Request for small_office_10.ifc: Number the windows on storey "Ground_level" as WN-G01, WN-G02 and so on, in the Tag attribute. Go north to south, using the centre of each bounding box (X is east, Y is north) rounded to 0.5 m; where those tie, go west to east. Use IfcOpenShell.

First a look at what the model holds.

```python
import ifcopenshell
import ifcopenshell.util.element
import ifcopenshell.util.placement

model = ifcopenshell.open("small_office_10.ifc")
print(model.schema)
storey = next(s for s in model.by_type("IfcBuildingStorey") if s.Name == "Ground_level")
windows = [e for e in ifcopenshell.util.element.get_decomposition(storey) if e.is_a("IfcWindow")]
for e in sorted(windows, key=lambda e: e.id()):
    origin = ifcopenshell.util.placement.get_local_placement(e.ObjectPlacement)[:3, 3]
    print(e.id(), e.Tag, e.Name, origin.round(2) + 0.0, sep=" | ")
```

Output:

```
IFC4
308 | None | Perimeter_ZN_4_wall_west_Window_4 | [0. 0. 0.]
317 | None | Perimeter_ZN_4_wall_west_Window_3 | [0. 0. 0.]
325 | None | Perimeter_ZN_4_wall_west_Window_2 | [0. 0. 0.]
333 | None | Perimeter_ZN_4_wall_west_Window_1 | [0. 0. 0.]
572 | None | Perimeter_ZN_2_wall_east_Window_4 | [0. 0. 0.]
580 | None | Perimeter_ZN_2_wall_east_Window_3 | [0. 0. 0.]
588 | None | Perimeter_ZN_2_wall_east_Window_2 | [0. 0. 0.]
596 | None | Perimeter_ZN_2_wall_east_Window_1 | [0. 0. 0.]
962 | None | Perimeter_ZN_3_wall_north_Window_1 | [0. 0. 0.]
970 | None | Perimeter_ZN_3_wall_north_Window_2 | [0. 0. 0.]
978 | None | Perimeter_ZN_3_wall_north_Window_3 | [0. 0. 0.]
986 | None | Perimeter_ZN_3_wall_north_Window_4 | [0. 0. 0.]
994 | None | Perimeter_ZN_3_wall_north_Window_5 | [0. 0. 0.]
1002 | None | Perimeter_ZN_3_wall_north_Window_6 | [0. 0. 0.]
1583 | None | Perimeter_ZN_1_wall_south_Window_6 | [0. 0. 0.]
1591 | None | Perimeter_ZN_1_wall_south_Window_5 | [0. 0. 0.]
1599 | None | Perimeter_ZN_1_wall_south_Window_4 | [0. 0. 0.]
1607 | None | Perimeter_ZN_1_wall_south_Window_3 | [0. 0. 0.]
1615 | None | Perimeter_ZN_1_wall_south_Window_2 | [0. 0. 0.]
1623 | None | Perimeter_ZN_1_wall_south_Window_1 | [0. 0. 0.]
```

```python
import ifcopenshell
import ifcopenshell.geom
import ifcopenshell.util.element
import ifcopenshell.util.shape

model = ifcopenshell.open("small_office_10.ifc")
settings = ifcopenshell.geom.settings()
settings.set("use-world-coords", True)


def centre(element):
    shape = ifcopenshell.geom.create_shape(settings, element)
    return ifcopenshell.util.shape.get_bbox_centroid(shape.geometry)


storey = next(s for s in model.by_type("IfcBuildingStorey") if s.Name == "Ground_level")
windows = [e for e in ifcopenshell.util.element.get_decomposition(storey) if e.is_a("IfcWindow")]

# Insertion points can sit at a corner or the storey origin, so sort by the geometry (in metres).
centres = {e: centre(e) for e in windows}
windows.sort(key=lambda e: (-round(centres[e][1] / 0.5), centres[e][0]))

for i, e in enumerate(windows, start=1):
    number = f"WN-G{i:02d}"
    e.Tag = number
    print(e.id(), number)

model.write("small_office_10_edited.ifc")
```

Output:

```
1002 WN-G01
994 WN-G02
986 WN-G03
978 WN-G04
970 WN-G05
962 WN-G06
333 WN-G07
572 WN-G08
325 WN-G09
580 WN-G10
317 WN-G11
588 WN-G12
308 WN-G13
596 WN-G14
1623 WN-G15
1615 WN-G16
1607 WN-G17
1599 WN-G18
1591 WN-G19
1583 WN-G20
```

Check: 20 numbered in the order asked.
